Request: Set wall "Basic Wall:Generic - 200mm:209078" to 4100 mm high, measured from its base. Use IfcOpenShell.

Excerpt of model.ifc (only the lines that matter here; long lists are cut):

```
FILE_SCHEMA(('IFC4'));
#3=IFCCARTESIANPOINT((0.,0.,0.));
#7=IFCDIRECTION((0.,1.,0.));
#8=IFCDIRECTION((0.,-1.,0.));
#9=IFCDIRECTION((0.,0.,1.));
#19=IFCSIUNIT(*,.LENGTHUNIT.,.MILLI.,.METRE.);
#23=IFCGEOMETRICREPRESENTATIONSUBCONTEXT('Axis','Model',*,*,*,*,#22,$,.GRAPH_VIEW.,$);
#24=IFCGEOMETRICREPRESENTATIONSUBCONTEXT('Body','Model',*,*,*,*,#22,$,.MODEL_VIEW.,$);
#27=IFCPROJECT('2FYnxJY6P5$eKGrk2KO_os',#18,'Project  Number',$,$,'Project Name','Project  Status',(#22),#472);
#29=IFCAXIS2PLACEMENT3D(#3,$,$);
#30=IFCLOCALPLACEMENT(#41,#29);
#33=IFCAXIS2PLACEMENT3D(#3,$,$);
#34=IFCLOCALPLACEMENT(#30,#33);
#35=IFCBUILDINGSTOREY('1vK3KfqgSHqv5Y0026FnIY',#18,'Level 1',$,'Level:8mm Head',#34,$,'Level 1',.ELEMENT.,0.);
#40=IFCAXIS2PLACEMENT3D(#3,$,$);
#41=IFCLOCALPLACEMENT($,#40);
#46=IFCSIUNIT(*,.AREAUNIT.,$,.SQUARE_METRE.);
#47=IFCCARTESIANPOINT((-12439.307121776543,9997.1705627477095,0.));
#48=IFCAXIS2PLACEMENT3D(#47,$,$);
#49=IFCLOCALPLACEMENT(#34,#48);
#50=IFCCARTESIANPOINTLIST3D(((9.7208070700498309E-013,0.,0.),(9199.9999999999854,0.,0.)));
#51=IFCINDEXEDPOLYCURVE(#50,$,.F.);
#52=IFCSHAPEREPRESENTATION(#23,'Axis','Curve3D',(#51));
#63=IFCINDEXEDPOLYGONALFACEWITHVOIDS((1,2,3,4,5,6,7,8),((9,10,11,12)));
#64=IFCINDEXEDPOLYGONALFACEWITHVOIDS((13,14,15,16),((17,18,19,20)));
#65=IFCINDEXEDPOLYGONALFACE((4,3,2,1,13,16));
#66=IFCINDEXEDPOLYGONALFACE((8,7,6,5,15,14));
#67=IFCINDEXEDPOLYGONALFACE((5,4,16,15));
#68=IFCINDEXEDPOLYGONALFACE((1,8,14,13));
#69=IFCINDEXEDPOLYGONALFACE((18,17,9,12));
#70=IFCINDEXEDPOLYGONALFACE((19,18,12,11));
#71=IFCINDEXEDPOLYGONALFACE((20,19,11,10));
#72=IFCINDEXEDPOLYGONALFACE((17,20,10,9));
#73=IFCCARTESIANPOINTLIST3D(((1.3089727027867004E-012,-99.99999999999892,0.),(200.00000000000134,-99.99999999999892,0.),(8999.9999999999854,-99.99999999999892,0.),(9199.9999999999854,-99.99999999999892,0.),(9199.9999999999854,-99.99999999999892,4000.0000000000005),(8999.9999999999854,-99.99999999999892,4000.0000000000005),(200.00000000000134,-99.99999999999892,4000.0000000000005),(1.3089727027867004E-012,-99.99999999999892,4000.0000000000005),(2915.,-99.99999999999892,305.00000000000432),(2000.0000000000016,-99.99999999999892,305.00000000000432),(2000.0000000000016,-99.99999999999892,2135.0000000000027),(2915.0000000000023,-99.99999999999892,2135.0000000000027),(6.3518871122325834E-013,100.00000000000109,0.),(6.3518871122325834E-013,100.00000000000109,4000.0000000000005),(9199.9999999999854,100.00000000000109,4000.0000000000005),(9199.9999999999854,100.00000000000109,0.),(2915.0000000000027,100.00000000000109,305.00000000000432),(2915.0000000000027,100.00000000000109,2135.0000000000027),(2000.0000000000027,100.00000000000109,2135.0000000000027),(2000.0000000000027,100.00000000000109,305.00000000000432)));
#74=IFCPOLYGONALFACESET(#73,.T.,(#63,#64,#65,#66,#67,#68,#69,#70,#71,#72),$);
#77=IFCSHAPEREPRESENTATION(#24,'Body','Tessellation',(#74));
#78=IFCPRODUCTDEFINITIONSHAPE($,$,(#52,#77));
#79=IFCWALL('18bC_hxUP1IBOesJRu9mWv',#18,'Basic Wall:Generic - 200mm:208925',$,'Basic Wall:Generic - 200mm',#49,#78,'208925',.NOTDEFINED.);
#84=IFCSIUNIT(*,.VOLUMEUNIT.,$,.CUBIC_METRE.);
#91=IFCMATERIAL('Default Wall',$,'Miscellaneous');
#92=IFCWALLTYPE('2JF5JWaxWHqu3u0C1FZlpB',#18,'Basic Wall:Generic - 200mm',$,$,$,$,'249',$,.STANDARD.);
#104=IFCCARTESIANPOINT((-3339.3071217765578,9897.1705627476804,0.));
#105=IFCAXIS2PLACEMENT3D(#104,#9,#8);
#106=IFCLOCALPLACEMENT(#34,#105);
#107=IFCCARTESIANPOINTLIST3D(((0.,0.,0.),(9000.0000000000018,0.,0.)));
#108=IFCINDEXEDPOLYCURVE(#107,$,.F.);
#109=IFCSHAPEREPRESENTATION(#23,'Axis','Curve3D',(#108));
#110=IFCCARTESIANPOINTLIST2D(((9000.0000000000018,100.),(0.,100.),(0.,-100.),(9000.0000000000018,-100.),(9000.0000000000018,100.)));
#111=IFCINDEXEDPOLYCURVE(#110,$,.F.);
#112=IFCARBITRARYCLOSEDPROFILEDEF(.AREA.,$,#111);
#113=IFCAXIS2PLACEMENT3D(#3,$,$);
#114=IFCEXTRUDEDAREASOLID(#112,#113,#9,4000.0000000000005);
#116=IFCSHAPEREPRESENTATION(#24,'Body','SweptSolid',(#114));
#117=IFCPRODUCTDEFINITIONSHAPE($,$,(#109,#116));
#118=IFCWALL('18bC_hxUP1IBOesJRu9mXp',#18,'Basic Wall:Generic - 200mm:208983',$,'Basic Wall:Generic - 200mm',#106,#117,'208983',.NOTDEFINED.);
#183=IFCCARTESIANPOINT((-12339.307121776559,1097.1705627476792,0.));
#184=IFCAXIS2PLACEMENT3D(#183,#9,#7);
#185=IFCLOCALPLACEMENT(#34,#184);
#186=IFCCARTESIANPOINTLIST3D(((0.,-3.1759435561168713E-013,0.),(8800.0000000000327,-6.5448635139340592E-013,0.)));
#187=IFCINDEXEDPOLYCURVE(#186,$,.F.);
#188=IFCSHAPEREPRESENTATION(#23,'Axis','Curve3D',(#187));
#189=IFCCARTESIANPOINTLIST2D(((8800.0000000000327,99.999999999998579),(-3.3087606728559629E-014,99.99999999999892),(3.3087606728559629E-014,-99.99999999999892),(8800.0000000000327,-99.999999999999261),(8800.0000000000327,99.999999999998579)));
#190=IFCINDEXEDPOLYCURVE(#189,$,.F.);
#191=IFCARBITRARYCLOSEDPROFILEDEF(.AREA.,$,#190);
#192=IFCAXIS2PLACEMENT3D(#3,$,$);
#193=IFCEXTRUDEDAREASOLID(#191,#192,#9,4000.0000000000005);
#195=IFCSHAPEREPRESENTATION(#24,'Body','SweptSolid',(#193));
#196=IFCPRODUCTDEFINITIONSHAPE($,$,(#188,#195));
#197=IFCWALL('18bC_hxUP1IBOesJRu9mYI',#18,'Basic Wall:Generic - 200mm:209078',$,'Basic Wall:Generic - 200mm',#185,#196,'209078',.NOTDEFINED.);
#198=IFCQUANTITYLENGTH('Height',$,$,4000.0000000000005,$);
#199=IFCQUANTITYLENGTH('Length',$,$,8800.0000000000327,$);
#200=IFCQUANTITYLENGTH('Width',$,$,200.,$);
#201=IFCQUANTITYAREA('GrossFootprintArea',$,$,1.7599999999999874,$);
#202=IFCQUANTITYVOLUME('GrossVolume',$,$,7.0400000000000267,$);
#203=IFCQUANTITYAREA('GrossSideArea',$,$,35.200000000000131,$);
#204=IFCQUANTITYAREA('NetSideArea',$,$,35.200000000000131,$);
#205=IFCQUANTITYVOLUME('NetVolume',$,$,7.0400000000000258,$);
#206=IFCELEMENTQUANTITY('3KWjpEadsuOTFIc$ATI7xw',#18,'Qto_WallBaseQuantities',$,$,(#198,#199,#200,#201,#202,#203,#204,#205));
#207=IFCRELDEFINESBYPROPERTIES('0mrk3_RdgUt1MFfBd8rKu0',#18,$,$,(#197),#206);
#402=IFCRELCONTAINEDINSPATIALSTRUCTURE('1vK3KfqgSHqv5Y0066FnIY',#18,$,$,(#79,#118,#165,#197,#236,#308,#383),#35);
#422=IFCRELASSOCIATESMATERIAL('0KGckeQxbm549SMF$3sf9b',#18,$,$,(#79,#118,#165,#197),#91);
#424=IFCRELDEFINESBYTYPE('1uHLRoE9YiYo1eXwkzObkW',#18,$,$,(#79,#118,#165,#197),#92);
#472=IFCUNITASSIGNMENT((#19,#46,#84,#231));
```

```python
import ifcopenshell
import ifcopenshell.api.pset
import ifcopenshell.geom
import ifcopenshell.util.element
import ifcopenshell.util.representation
import ifcopenshell.util.shape
import ifcopenshell.util.unit

model = ifcopenshell.open("model.ifc")
unit_scale = ifcopenshell.util.unit.calculate_unit_scale(model)
area_scale = ifcopenshell.util.unit.calculate_unit_scale(model, "AREAUNIT")
volume_scale = ifcopenshell.util.unit.calculate_unit_scale(model, "VOLUMEUNIT")
settings = ifcopenshell.geom.settings()


def volume(element):
    """Net volume in cubic metres, openings subtracted."""
    shape = ifcopenshell.geom.create_shape(settings, element)
    return ifcopenshell.util.shape.get_volume(shape.geometry)


wall = model.by_guid("18bC_hxUP1IBOesJRu9mYI")
before = volume(wall)

body = ifcopenshell.util.representation.get_representation(wall, "Model", "Body")
solid = body.Items[0]
old_height = solid.Depth
solid.Depth = 4.1 / unit_scale
after = volume(wall)
thickness = 0.2  # wall thickness in metres

# Update the stored height, areas and volumes.
qto = model.by_id(ifcopenshell.util.element.get_pset(wall, "Qto_WallBaseQuantities", should_inherit=False)["id"])
ifcopenshell.api.pset.edit_qto(model, qto=qto, properties={
    "Height": solid.Depth,
    "GrossVolume": ifcopenshell.util.element.get_pset(wall, "Qto_WallBaseQuantities", "GrossVolume") * solid.Depth / old_height,
    "GrossSideArea": ifcopenshell.util.element.get_pset(wall, "Qto_WallBaseQuantities", "GrossSideArea") * solid.Depth / old_height,
    "NetSideArea": after / thickness / area_scale,
    "NetVolume": after / volume_scale,
})

print(f"height {old_height:g} -> {solid.Depth:g}, volume {before:.3f} -> {after:.3f} m3")

model.write("model_rev.ifc")
```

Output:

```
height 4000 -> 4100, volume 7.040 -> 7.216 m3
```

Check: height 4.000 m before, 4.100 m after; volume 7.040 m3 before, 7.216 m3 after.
